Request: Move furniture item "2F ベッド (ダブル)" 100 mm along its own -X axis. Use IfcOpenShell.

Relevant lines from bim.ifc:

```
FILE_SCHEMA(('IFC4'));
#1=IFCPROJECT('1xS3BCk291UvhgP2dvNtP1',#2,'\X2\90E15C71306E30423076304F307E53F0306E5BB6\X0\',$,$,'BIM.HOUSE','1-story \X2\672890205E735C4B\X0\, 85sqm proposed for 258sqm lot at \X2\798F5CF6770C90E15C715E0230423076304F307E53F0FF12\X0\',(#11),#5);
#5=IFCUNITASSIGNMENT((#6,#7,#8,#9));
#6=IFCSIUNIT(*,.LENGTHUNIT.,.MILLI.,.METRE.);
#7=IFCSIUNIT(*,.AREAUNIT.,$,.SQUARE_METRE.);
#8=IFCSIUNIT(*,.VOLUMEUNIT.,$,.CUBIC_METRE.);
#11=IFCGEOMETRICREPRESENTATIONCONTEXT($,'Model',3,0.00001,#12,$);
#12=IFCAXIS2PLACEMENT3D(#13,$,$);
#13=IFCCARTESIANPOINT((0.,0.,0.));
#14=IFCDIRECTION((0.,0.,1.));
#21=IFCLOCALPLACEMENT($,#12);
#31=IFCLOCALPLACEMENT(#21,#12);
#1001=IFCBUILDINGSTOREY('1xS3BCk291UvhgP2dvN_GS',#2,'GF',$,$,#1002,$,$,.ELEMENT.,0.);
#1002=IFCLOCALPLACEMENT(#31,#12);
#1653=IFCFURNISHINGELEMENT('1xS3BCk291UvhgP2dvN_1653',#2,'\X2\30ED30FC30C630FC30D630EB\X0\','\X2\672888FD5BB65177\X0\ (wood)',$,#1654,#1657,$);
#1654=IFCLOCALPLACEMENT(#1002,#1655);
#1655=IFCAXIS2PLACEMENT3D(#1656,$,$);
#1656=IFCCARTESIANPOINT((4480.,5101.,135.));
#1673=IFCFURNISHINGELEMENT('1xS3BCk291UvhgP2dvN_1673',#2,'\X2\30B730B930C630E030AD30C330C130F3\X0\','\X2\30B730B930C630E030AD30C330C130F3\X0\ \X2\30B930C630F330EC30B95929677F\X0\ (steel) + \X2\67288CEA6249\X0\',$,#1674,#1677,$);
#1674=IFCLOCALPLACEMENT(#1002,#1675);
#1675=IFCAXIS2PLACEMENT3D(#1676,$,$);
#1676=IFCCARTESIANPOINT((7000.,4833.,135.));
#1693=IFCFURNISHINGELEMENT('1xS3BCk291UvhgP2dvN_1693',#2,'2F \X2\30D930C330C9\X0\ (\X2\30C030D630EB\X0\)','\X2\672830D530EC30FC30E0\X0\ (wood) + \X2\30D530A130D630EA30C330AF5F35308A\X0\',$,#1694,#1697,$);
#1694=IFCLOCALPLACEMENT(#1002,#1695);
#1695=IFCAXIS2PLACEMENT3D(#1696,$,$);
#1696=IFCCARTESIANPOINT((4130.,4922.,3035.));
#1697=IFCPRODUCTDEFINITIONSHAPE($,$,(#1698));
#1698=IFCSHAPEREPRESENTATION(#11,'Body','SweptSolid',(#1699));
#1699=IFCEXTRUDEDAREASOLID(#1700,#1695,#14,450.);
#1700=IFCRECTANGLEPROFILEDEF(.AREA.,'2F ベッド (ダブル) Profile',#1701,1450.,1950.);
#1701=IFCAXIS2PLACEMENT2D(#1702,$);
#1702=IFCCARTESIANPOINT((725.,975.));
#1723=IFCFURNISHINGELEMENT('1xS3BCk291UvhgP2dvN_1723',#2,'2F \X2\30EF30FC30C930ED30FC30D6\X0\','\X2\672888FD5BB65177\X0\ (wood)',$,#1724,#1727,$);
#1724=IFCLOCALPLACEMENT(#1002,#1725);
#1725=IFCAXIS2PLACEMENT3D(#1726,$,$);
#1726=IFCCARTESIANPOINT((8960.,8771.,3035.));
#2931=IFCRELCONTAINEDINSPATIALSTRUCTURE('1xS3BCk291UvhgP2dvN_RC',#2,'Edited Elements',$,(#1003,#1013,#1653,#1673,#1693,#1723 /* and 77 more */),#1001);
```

```python
import ifcopenshell
import ifcopenshell.api.geometry
import ifcopenshell.util.placement
import ifcopenshell.util.unit

model = ifcopenshell.open("bim.ifc")
unit_scale = ifcopenshell.util.unit.calculate_unit_scale(model)

item = model.by_id(1693)
matrix = ifcopenshell.util.placement.get_local_placement(item.ObjectPlacement)
matrix[:3, 3] -= matrix[:3, 0] * 0.1 / unit_scale
ifcopenshell.api.geometry.edit_object_placement(model, product=item, matrix=matrix, is_si=False)

print(ifcopenshell.util.placement.get_local_placement(item.ObjectPlacement).round(3) + 0.0)

model.write("bim_updated.ifc")
```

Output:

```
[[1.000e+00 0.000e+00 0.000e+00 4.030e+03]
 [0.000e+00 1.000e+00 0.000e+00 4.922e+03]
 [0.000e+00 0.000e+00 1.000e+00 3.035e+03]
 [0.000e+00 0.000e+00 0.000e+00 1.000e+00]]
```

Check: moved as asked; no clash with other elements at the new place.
